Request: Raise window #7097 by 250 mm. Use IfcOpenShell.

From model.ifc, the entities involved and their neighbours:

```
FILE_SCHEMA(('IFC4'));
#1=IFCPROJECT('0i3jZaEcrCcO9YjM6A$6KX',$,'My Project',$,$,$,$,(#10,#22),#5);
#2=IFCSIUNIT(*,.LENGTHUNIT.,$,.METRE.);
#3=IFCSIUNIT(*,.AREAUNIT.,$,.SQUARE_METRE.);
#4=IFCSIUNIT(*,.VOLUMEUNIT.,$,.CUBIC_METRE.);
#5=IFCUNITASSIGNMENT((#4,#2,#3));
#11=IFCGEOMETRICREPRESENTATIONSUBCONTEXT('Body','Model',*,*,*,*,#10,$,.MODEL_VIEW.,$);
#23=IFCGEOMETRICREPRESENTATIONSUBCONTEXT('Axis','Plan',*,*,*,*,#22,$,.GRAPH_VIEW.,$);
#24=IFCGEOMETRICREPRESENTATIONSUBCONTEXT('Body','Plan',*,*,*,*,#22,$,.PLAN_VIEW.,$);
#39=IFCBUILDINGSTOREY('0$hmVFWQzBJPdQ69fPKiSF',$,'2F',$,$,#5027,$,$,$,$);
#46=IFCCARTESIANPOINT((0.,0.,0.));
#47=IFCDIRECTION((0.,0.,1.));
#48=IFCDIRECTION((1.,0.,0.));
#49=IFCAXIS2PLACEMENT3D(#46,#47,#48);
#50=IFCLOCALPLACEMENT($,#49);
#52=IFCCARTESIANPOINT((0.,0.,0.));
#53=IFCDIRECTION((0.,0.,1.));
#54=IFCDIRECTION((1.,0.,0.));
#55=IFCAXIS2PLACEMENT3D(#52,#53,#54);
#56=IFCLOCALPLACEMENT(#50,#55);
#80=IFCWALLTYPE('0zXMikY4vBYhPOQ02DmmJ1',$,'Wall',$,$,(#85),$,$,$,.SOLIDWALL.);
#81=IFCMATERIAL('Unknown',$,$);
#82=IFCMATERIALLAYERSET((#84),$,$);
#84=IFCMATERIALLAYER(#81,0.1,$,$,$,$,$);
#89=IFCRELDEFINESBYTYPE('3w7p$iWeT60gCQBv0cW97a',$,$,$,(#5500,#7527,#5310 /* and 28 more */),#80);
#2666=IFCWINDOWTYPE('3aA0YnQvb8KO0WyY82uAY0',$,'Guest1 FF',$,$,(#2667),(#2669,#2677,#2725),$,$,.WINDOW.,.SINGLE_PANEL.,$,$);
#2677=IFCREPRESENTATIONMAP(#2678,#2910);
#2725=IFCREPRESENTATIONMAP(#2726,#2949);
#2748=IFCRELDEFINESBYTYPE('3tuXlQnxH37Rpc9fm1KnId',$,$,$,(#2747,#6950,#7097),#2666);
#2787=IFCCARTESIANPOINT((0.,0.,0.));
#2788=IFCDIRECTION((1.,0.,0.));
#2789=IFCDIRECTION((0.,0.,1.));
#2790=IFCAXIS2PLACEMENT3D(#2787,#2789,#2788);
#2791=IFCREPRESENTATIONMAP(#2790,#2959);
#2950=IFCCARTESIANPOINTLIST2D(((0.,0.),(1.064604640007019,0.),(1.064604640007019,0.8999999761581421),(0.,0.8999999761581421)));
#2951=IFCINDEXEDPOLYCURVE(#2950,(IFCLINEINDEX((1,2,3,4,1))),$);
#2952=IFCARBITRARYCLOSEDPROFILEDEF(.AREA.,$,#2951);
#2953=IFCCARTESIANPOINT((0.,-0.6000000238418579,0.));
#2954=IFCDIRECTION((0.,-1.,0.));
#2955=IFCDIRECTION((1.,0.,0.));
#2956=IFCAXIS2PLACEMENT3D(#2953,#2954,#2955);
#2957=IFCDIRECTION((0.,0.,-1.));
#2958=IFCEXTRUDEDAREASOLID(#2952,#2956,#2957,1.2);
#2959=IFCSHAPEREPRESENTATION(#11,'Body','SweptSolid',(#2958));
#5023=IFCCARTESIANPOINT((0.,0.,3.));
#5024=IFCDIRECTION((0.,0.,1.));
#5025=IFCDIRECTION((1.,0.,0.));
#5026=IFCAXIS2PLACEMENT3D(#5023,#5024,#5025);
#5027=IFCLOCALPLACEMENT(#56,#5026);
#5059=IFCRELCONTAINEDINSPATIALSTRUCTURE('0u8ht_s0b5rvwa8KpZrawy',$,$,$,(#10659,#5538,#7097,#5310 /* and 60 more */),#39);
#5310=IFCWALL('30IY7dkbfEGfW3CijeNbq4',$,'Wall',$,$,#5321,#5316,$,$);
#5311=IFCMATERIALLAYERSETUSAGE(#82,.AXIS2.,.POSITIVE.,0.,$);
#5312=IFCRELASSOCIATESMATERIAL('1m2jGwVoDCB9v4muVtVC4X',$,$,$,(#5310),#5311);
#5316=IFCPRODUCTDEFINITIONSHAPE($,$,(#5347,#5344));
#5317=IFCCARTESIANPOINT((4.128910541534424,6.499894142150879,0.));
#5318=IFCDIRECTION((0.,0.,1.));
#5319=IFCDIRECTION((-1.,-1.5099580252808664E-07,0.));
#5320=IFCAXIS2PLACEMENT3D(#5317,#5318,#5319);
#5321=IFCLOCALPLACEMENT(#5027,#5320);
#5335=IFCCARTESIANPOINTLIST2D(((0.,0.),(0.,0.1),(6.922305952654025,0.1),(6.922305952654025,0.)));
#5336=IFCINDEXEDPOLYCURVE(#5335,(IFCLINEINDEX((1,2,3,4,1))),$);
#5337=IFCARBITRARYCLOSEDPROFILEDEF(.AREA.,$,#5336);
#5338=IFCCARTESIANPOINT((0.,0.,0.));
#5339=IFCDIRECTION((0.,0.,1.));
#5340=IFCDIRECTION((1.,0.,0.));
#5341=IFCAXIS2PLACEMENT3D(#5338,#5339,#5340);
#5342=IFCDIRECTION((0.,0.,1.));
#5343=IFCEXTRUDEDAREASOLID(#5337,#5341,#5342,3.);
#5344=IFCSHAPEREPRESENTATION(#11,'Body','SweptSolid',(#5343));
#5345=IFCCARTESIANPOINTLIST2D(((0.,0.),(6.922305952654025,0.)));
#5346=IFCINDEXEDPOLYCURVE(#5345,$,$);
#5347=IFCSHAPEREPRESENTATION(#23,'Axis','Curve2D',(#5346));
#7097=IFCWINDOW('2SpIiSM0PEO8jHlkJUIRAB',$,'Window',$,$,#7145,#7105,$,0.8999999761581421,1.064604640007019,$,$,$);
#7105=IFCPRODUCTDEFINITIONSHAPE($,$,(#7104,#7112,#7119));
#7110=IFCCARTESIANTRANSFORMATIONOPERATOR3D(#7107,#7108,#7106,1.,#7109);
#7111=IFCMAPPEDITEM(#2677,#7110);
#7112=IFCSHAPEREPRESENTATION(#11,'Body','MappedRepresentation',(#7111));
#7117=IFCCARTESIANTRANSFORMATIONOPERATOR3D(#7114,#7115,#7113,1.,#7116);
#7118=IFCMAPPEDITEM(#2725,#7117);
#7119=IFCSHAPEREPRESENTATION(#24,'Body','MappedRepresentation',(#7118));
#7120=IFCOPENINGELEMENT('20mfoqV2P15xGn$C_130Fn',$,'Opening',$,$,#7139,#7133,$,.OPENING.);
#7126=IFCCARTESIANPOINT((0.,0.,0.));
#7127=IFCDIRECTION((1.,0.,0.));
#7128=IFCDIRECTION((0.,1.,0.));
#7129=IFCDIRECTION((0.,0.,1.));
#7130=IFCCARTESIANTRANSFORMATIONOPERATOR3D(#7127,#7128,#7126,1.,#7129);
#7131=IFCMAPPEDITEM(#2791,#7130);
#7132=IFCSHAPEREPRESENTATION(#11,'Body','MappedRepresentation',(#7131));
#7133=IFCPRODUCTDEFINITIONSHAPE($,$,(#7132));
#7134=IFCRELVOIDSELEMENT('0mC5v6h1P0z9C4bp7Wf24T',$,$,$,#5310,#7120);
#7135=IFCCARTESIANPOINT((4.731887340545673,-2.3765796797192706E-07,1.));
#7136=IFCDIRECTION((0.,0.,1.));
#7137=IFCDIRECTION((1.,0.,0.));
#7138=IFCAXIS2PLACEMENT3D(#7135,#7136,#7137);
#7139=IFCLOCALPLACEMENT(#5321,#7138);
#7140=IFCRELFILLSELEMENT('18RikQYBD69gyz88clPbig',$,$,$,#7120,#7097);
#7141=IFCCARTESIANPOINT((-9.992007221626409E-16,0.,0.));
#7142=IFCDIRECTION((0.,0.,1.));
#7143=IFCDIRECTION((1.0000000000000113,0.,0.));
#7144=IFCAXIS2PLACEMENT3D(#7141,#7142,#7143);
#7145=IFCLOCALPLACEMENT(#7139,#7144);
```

```python
import numpy as np
import ifcopenshell
import ifcopenshell.api.geometry
import ifcopenshell.util.placement
import ifcopenshell.util.unit

model = ifcopenshell.open("model.ifc")
unit_scale = ifcopenshell.util.unit.calculate_unit_scale(model)

window = model.by_id(7097)
opening = window.FillsVoids[0].RelatingOpeningElement
dz = 0.25 / unit_scale

shift = np.array([0.0, 0.0, dz])
# The window is placed relative to its opening, so it follows when the opening moves.
matrix = ifcopenshell.util.placement.get_local_placement(opening.ObjectPlacement)
matrix[:3, 3] += shift
ifcopenshell.api.geometry.edit_object_placement(
    model, product=opening, matrix=matrix, is_si=False, should_transform_children=True
)

print(f"moved by {dz * unit_scale:+.3f} m")

model.write("model_edited.ifc")
```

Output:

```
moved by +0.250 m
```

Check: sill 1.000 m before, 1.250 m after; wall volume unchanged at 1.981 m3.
